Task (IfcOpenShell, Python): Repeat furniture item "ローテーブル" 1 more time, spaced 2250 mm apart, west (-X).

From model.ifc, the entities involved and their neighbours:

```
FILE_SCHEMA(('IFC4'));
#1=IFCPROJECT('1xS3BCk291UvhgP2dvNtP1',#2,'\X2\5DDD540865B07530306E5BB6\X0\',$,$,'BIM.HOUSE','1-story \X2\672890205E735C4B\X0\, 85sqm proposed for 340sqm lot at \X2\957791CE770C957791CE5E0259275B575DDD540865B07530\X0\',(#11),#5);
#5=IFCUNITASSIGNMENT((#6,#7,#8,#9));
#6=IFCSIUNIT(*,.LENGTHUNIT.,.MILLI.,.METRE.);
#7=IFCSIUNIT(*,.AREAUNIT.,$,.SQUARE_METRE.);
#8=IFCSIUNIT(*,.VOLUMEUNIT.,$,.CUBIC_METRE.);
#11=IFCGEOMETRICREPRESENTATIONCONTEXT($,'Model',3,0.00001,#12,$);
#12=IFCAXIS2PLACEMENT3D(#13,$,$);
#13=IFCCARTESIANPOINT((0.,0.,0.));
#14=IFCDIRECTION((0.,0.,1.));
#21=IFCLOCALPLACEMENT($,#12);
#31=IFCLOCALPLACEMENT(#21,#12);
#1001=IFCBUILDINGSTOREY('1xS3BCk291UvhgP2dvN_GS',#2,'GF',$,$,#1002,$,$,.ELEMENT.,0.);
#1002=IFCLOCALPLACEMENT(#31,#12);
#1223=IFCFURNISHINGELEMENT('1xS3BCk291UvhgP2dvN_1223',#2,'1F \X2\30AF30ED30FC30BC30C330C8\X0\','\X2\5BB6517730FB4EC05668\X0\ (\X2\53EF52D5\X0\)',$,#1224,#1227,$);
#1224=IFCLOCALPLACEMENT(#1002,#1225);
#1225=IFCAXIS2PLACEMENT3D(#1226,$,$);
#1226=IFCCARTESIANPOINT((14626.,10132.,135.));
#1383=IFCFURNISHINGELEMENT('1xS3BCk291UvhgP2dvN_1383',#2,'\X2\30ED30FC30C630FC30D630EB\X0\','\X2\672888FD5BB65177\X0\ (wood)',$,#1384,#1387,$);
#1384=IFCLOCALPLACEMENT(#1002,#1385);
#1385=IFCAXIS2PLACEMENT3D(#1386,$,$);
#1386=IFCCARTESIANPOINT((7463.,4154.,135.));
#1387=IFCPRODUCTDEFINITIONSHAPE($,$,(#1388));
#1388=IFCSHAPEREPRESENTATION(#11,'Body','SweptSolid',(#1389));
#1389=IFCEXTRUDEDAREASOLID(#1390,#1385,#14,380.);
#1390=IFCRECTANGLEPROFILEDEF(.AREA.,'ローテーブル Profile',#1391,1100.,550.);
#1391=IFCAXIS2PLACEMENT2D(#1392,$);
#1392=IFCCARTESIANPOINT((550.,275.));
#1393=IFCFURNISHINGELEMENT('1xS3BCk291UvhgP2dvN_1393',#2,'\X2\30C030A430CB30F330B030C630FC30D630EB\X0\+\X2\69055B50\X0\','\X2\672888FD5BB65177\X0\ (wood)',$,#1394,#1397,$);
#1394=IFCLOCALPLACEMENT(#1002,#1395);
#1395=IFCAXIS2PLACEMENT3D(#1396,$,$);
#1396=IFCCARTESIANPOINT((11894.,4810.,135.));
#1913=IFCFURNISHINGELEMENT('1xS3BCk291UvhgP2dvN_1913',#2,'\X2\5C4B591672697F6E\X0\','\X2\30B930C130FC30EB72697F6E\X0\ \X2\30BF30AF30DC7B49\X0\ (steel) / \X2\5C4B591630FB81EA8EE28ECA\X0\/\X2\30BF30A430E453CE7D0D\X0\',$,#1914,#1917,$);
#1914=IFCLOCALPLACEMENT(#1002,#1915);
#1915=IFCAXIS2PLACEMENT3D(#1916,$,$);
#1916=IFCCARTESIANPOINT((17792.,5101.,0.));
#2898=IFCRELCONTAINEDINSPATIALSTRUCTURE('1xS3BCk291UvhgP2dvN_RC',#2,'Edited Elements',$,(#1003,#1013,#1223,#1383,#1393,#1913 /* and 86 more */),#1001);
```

```python
import numpy as np
import ifcopenshell
import ifcopenshell.api.geometry
import ifcopenshell.api.root
import ifcopenshell.util.element
import ifcopenshell.util.placement
import ifcopenshell.util.unit

model = ifcopenshell.open("model.ifc")
unit_scale = ifcopenshell.util.unit.calculate_unit_scale(model)


def reuse_history(source, copy):
    """copy_class also copies each property set's owner history, people and application; keep the originals."""
    for rel in copy.IsDefinedBy:
        if rel.is_a("IfcRelDefinesByProperties") and (history := rel.RelatingPropertyDefinition.OwnerHistory):
            rel.RelatingPropertyDefinition.OwnerHistory = source.OwnerHistory
            ifcopenshell.util.element.remove_deep2(model, history)


source = model.by_guid("1xS3BCk291UvhgP2dvN_1383")
base = ifcopenshell.util.placement.get_local_placement(source.ObjectPlacement)
step = np.array([-1.0, 0.0, 0.0]) * 2.25 / unit_scale

for i in range(1, 2):
    copy = ifcopenshell.api.root.copy_class(model, product=source)
    copy.Representation = ifcopenshell.util.element.copy_deep(
        model, source.Representation, exclude=["IfcGeometricRepresentationContext", "IfcRepresentationMap"]
    )
    reuse_history(source, copy)
    matrix = base.copy()
    matrix[:3, 3] += i * step
    print("added at", matrix[:3, 3].round(3) + 0.0)
    ifcopenshell.api.geometry.edit_object_placement(model, product=copy, matrix=matrix, is_si=False)

model.write("model-out.ifc")
```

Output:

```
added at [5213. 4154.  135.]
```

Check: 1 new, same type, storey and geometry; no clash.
